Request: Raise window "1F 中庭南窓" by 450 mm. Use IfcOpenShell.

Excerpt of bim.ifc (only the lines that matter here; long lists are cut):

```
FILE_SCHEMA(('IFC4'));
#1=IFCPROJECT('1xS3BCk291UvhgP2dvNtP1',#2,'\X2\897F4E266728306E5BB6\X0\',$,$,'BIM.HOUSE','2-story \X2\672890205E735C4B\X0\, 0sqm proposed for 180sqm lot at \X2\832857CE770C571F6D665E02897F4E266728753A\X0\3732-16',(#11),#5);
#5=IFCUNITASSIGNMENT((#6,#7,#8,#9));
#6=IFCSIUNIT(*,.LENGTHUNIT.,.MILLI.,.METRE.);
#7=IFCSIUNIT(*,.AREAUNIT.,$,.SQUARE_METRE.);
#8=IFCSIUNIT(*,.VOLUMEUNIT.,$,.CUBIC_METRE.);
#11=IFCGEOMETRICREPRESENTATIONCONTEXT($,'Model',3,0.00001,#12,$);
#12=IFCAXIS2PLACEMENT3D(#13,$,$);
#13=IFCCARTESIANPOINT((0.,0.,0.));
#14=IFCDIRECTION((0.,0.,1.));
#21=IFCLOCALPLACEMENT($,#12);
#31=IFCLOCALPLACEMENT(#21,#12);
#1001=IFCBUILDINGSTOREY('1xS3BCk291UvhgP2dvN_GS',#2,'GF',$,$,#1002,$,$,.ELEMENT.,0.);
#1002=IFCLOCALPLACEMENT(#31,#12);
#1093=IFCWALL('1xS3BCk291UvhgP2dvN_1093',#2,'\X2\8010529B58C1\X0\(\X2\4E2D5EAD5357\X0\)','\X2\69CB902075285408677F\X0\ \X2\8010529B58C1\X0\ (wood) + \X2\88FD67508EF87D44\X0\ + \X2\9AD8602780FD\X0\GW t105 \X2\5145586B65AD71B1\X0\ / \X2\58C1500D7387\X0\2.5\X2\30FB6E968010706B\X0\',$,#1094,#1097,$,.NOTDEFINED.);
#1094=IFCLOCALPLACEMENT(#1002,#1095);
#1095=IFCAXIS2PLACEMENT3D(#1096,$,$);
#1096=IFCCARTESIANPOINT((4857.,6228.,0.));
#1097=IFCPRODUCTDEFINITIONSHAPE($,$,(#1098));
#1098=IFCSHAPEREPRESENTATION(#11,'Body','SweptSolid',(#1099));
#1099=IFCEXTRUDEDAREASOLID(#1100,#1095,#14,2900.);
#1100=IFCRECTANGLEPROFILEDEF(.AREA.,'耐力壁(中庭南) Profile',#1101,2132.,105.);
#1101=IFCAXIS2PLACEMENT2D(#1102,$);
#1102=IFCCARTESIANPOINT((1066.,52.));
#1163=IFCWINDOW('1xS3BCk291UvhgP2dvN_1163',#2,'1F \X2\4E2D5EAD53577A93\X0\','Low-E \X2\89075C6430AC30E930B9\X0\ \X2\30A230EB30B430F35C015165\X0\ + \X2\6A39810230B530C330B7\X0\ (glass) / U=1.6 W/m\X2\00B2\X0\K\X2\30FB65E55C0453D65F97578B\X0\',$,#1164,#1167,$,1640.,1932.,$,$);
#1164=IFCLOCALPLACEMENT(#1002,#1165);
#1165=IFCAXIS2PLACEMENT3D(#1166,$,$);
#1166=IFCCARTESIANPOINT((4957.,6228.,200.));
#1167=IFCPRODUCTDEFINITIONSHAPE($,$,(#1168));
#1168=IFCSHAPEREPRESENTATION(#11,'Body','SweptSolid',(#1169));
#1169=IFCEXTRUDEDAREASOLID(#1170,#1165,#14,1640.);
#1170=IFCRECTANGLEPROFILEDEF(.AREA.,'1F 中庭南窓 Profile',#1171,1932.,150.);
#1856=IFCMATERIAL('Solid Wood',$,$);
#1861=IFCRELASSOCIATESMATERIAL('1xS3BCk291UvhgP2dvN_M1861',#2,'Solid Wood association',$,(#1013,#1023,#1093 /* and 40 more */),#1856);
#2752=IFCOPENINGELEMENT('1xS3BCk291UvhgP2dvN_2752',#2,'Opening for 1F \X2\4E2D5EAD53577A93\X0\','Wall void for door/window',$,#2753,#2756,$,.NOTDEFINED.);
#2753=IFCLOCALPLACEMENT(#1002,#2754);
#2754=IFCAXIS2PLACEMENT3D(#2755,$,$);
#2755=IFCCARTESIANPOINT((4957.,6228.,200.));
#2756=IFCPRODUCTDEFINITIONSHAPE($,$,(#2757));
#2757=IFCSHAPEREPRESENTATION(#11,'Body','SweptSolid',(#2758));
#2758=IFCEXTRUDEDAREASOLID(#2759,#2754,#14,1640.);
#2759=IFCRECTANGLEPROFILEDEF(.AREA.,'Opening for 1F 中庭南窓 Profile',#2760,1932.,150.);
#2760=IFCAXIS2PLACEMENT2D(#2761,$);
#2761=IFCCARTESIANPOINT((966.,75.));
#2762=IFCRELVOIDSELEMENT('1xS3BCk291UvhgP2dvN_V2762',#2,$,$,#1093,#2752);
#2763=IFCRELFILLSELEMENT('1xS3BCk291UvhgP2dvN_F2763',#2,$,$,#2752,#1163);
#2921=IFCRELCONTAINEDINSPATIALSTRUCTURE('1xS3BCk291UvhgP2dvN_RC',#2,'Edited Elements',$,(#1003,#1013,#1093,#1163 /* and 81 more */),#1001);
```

```python
import numpy as np
import ifcopenshell
import ifcopenshell.api.geometry
import ifcopenshell.util.placement
import ifcopenshell.util.unit

model = ifcopenshell.open("bim.ifc")
unit_scale = ifcopenshell.util.unit.calculate_unit_scale(model)

window = model.by_guid("1xS3BCk291UvhgP2dvN_1163")
opening = window.FillsVoids[0].RelatingOpeningElement
dz = 450.0

shift = np.array([0.0, 0.0, dz])
# The window is not placed relative to its opening, so move both.
for product in (opening, window):
    matrix = ifcopenshell.util.placement.get_local_placement(product.ObjectPlacement)
    matrix[:3, 3] += shift
    ifcopenshell.api.geometry.edit_object_placement(model, product=product, matrix=matrix, is_si=False)

print(f"moved by {dz * unit_scale:+.3f} m")

model.write("bim_v2.ifc")
```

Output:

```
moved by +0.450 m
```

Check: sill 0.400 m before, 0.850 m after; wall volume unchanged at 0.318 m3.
